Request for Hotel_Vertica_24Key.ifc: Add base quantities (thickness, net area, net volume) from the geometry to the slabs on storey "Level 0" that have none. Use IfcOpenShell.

First a look at what the model holds.

```python
import ifcopenshell
import ifcopenshell.util.element
import ifcopenshell.util.unit

model = ifcopenshell.open("Hotel_Vertica_24Key.ifc")
print(model.schema)
for unit_type in ("LENGTHUNIT", "AREAUNIT", "VOLUMEUNIT"):
    print(unit_type, ifcopenshell.util.unit.calculate_unit_scale(model, unit_type))
storey = next(s for s in model.by_type("IfcBuildingStorey") if s.Name == "Level 0")
slabs = [e for e in ifcopenshell.util.element.get_decomposition(storey) if e.is_a("IfcSlab")]
for e in sorted(slabs, key=lambda e: e.id()):
    print(e.id(), e.is_a(), e.Name, list(ifcopenshell.util.element.get_psets(e, qtos_only=True)), sep=" | ")
```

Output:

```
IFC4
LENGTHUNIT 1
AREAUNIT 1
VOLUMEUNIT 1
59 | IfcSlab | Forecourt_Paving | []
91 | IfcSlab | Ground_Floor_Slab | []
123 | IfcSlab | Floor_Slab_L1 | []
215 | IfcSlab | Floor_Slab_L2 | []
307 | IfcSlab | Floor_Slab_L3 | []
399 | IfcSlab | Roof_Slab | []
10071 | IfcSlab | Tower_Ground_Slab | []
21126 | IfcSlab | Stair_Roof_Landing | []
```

```python
import ifcopenshell
import ifcopenshell.api.pset
import ifcopenshell.geom
import ifcopenshell.util.element
import ifcopenshell.util.shape
import ifcopenshell.util.unit

model = ifcopenshell.open("Hotel_Vertica_24Key.ifc")
unit_scale = ifcopenshell.util.unit.calculate_unit_scale(model)
area_scale = ifcopenshell.util.unit.calculate_unit_scale(model, "AREAUNIT")
volume_scale = ifcopenshell.util.unit.calculate_unit_scale(model, "VOLUMEUNIT")
settings = ifcopenshell.geom.settings()

storey = next(s for s in model.by_type("IfcBuildingStorey") if s.Name == "Level 0")
slabs = [e for e in ifcopenshell.util.element.get_decomposition(storey) if e.is_a("IfcSlab")]

for e in sorted(slabs, key=lambda e: e.id()):
    if ifcopenshell.util.element.get_psets(e, qtos_only=True, should_inherit=False):
        continue
    # Geometry comes back in metres, in the element's own axes.
    shape = ifcopenshell.geom.create_shape(settings, e)
    values = {
        "Width": ifcopenshell.util.shape.get_z(shape.geometry) / unit_scale,
        "NetArea": ifcopenshell.util.shape.get_footprint_area(shape.geometry) / area_scale,
        "NetVolume": ifcopenshell.util.shape.get_volume(shape.geometry) / volume_scale,
    }
    qto = ifcopenshell.api.pset.add_qto(model, product=e, name="Qto_SlabBaseQuantities")
    ifcopenshell.api.pset.edit_qto(model, qto=qto, properties=values)
    print(e.id(), {k: round(v, 3) for k, v in values.items()})

model.write("Hotel_Vertica_24Key_updated.ifc")
```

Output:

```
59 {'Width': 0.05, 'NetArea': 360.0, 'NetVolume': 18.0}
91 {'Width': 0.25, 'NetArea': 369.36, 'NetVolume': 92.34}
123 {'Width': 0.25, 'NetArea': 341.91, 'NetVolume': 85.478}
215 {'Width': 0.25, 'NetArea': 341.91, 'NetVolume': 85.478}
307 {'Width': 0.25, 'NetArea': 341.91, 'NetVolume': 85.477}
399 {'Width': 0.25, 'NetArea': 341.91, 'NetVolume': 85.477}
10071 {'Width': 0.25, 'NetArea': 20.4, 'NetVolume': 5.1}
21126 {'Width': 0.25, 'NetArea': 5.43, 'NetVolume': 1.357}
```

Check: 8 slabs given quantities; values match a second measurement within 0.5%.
